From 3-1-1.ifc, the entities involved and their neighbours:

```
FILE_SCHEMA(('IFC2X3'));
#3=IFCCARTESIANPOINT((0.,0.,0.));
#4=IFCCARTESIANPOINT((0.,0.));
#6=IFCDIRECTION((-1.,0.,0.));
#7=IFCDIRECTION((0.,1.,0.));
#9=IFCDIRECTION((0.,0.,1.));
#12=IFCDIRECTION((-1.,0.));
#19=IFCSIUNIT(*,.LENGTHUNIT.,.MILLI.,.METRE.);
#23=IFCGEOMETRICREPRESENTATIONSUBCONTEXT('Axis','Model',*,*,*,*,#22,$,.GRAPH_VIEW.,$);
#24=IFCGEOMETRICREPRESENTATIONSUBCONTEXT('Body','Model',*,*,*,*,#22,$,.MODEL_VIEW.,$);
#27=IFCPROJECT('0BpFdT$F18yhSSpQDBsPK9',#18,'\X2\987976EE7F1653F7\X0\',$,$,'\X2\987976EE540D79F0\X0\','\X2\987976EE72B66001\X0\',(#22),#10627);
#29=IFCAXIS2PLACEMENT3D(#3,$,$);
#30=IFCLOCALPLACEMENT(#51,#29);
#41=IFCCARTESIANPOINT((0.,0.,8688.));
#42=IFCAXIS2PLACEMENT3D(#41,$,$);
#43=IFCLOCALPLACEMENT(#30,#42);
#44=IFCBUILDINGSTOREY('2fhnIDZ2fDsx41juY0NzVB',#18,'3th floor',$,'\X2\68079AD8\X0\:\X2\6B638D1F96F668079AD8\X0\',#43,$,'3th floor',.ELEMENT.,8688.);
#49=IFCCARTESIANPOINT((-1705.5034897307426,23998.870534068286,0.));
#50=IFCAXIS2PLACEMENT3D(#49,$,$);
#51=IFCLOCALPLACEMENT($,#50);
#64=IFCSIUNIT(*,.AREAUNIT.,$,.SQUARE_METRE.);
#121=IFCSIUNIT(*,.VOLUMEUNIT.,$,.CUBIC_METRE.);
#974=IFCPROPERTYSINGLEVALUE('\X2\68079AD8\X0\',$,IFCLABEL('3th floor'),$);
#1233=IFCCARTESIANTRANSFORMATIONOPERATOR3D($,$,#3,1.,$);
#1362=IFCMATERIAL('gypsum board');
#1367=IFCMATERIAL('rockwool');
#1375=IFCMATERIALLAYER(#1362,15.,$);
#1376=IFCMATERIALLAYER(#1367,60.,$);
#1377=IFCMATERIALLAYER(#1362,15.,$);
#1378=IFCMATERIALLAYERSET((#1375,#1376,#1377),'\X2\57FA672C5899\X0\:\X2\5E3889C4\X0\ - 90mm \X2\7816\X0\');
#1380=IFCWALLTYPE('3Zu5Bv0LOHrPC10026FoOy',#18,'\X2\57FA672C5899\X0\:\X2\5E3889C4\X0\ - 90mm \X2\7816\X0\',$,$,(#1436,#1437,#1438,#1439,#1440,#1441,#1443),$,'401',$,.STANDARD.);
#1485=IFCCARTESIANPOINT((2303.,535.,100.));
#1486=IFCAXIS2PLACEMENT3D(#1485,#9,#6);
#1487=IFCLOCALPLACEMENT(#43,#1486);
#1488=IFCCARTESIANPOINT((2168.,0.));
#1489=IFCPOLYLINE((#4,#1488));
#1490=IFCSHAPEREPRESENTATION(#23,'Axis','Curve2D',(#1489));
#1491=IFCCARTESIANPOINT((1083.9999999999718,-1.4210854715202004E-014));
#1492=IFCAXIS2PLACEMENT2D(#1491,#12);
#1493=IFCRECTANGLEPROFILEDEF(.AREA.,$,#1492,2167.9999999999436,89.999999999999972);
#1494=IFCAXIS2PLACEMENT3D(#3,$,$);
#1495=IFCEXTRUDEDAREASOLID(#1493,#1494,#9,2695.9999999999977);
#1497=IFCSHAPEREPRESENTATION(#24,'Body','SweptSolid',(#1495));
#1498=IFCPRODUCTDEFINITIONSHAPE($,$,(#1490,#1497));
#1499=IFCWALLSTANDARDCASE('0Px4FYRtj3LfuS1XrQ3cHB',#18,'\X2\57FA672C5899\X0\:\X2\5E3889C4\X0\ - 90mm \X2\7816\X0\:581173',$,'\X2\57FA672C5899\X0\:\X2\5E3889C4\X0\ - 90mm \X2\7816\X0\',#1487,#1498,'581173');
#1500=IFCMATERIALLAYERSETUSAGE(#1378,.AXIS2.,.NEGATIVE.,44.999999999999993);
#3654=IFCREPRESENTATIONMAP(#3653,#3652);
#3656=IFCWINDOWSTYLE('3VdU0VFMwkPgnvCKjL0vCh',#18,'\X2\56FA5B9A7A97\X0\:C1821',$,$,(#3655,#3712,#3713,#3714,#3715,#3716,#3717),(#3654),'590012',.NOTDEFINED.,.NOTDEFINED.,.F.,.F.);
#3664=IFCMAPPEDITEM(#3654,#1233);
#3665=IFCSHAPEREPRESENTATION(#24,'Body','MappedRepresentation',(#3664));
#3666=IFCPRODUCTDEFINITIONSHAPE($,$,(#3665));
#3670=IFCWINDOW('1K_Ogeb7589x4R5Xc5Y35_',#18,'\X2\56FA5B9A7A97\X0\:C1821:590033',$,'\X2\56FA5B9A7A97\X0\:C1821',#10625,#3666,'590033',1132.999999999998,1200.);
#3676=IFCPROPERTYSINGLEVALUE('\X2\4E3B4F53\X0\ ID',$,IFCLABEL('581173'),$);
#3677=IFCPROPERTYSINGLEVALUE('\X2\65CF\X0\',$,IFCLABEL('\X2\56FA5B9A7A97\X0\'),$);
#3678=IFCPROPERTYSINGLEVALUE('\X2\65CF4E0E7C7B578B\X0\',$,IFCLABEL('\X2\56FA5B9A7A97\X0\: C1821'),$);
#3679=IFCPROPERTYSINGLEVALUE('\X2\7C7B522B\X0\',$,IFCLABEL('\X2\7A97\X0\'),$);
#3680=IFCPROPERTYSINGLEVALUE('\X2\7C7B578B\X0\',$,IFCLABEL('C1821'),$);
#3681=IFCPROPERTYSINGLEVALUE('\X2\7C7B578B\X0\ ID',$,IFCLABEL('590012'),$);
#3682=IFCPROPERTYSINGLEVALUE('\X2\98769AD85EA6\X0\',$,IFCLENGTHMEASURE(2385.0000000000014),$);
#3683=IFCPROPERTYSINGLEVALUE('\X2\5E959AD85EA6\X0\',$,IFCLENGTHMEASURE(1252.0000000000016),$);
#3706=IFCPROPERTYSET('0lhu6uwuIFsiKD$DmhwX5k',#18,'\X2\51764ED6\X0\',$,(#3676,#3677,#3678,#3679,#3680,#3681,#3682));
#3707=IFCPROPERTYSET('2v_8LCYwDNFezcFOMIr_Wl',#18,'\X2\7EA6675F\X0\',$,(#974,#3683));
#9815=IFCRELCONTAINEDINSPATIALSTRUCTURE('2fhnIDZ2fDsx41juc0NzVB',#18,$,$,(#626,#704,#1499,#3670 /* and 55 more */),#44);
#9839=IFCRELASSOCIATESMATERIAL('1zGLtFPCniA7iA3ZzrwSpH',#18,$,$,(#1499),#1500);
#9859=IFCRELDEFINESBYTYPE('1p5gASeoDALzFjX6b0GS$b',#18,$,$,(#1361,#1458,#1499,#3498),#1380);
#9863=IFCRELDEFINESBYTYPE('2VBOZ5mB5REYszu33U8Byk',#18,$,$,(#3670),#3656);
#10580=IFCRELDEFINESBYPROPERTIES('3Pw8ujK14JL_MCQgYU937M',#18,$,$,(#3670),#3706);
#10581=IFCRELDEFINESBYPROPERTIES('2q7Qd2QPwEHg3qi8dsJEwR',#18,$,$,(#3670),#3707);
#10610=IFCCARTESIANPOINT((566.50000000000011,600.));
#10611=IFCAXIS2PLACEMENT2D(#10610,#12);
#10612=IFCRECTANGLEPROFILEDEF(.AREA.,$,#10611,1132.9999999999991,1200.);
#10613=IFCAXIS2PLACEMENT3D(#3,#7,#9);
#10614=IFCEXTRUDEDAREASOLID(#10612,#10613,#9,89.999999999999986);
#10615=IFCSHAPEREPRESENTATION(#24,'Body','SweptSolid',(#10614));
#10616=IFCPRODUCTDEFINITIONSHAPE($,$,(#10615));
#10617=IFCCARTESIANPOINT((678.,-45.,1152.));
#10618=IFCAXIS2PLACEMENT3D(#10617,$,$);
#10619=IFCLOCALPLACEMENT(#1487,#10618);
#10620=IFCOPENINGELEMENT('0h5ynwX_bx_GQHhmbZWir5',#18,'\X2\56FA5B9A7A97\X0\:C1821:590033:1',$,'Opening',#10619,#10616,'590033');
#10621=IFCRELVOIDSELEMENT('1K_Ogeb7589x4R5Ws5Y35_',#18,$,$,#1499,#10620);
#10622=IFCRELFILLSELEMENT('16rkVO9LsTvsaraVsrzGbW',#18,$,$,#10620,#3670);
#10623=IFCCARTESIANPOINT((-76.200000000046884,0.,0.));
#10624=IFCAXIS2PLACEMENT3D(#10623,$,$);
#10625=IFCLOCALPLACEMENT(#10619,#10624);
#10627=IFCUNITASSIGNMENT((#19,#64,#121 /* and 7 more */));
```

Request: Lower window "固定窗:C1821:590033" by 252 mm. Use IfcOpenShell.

```python
import numpy as np
import ifcopenshell
import ifcopenshell.api.geometry
import ifcopenshell.api.pset
import ifcopenshell.util.element
import ifcopenshell.util.placement
import ifcopenshell.util.unit

model = ifcopenshell.open("3-1-1.ifc")
unit_scale = ifcopenshell.util.unit.calculate_unit_scale(model)

window = model.by_guid("1K_Ogeb7589x4R5Xc5Y35_")
opening = window.FillsVoids[0].RelatingOpeningElement
dz = -0.252 / unit_scale

shift = np.array([0.0, 0.0, dz])
# The window is placed relative to its opening, so it follows when the opening moves.
matrix = ifcopenshell.util.placement.get_local_placement(opening.ObjectPlacement)
matrix[:3, 3] += shift
ifcopenshell.api.geometry.edit_object_placement(
    model, product=opening, matrix=matrix, is_si=False, should_transform_children=True
)

# Keep the stored heights in step.
pset = model.by_id(ifcopenshell.util.element.get_pset(window, "其他", should_inherit=False)["id"])
ifcopenshell.api.pset.edit_pset(model, pset=pset, properties={
    "顶高度": model.create_entity("IfcLengthMeasure", ifcopenshell.util.element.get_pset(window, "其他", "顶高度") + dz),
})
pset = model.by_id(ifcopenshell.util.element.get_pset(window, "约束", should_inherit=False)["id"])
ifcopenshell.api.pset.edit_pset(model, pset=pset, properties={
    "底高度": model.create_entity("IfcLengthMeasure", ifcopenshell.util.element.get_pset(window, "约束", "底高度") + dz),
})

print(f"moved by {dz * unit_scale:+.3f} m")

model.write("3-1-1_edited.ifc")
```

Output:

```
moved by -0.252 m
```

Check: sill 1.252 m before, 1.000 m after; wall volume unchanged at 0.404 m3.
